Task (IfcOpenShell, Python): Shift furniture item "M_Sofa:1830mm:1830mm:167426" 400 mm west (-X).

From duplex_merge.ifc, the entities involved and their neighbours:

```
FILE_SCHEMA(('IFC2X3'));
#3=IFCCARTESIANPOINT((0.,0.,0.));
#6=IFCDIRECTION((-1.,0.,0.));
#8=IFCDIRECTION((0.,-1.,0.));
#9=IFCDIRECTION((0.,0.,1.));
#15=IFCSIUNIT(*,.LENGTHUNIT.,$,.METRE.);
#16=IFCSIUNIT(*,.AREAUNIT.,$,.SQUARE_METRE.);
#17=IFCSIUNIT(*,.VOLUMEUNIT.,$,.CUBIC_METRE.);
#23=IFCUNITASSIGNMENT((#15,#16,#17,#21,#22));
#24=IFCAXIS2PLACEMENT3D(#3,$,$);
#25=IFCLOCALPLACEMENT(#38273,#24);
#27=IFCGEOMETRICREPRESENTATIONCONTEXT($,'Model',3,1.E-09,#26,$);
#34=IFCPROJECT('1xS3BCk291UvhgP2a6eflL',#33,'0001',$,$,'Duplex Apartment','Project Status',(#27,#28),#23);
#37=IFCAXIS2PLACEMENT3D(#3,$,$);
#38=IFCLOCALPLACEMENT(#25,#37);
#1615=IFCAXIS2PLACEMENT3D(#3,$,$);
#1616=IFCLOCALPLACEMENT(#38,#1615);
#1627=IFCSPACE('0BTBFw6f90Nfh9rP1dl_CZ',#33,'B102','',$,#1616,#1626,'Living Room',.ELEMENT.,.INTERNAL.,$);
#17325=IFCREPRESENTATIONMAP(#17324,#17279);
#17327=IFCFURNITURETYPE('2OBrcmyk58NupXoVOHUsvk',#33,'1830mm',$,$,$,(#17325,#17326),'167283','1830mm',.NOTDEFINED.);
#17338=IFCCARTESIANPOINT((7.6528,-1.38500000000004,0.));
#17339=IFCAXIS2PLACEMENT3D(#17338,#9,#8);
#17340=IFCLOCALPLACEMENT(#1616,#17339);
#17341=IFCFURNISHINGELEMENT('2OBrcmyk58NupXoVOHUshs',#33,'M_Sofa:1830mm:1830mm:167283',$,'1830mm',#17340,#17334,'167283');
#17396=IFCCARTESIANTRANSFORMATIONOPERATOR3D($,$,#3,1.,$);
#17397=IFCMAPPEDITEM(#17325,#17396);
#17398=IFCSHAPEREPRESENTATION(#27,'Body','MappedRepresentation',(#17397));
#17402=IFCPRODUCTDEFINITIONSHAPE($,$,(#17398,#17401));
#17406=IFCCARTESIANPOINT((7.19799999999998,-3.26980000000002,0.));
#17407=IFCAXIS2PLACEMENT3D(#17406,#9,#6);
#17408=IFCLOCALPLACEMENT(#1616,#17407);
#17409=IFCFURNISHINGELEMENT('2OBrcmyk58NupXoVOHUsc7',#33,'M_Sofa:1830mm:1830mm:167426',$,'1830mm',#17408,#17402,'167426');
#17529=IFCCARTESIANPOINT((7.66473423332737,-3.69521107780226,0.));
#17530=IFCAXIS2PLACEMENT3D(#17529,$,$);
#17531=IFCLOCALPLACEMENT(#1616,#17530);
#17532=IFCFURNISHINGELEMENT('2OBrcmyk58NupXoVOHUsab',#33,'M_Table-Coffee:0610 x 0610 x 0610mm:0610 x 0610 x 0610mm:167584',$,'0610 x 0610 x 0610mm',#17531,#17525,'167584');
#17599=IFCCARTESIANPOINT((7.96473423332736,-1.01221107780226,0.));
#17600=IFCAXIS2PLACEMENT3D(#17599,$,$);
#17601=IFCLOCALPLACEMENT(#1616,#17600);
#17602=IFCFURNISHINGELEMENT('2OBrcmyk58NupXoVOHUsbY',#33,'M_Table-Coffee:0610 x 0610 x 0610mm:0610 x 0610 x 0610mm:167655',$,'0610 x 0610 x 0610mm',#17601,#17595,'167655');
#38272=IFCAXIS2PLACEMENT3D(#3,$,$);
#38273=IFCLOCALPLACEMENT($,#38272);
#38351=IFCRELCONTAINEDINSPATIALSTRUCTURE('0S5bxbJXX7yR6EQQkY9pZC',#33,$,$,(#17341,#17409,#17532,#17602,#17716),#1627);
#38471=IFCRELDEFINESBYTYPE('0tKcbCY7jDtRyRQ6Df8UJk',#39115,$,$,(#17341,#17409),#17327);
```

```python
import ifcopenshell
import ifcopenshell.api.geometry
import ifcopenshell.util.placement

model = ifcopenshell.open("duplex_merge.ifc")

item = model.by_id(17409)
matrix = ifcopenshell.util.placement.get_local_placement(item.ObjectPlacement)
matrix[0, 3] -= 0.4
ifcopenshell.api.geometry.edit_object_placement(model, product=item, matrix=matrix, is_si=False)

print(ifcopenshell.util.placement.get_local_placement(item.ObjectPlacement).round(3) + 0.0)

model.write("duplex_merge_rev.ifc")
```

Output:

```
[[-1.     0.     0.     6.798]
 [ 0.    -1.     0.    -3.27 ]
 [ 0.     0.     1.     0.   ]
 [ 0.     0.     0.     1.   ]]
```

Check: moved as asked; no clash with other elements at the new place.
